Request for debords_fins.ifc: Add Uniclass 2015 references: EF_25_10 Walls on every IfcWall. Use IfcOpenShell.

First a look at what the model holds.

```python
import ifcopenshell

model = ifcopenshell.open("debords_fins.ifc")
print(model.schema)
print("classifications:", [c.Name for c in model.by_type("IfcClassification")])
for ifc_class in ("IfcDoor", "IfcRoof", "IfcStair", "IfcWall", "IfcWindow"):
    print(ifc_class, len(model.by_type(ifc_class)))
```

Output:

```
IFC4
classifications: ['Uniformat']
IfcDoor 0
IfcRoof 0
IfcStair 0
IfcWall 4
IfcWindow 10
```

```python
import ifcopenshell
import ifcopenshell.api.classification

model = ifcopenshell.open("debords_fins.ifc")

system = ifcopenshell.api.classification.add_classification(model, classification="Uniclass 2015")

codes = {
    "IfcWall": ("EF_25_10", "Walls"),
}
for ifc_class, (code, name) in codes.items():
    products = model.by_type(ifc_class)
    ifcopenshell.api.classification.add_reference(
        model, products=products, classification=system, identification=code, name=name
    )
    print(code, len(products))

model.write("debords_fins_v2.ifc")
```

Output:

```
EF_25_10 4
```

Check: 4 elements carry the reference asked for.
